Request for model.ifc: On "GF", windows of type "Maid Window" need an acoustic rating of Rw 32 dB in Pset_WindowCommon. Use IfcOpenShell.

First a look at what the model holds.

```python
import ifcopenshell
import ifcopenshell.util.element

model = ifcopenshell.open("model.ifc")
print(model.schema)
storey = next(s for s in model.by_type("IfcBuildingStorey") if s.Name == "GF")
windows = [e for e in ifcopenshell.util.element.get_decomposition(storey) if e.is_a("IfcWindow")]
seen = {}
for e in windows:
    element_type = ifcopenshell.util.element.get_type(e)
    key = (element_type.Name if element_type != e and element_type else None, ifcopenshell.util.element.get_pset(e, "Pset_WindowCommon", "AcousticRating"))
    seen[key] = seen.get(key, 0) + 1
for (name, value), count in sorted(seen.items(), key=str):
    print(count, "x", name, "|", value)
```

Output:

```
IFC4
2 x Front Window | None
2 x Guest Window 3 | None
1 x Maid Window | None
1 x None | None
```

```python
import ifcopenshell
import ifcopenshell.api.pset
import ifcopenshell.util.element

model = ifcopenshell.open("model.ifc")

storey = next(s for s in model.by_type("IfcBuildingStorey") if s.Name == "GF")
windows = [e for e in ifcopenshell.util.element.get_decomposition(storey) if e.is_a("IfcWindow")]

count = 0
for e in windows:
    element_type = ifcopenshell.util.element.get_type(e)
    if element_type in (None, e) or element_type.Name != "Maid Window":
        continue
    # add_pset returns the element's existing set when there is one.
    pset = ifcopenshell.api.pset.add_pset(model, product=e, name="Pset_WindowCommon")
    ifcopenshell.api.pset.edit_pset(model, pset=pset, properties={"AcousticRating": "Rw 32 dB"})
    count += 1

print(count, "windows updated")

model.write("model_edited.ifc")
```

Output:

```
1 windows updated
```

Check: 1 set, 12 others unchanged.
